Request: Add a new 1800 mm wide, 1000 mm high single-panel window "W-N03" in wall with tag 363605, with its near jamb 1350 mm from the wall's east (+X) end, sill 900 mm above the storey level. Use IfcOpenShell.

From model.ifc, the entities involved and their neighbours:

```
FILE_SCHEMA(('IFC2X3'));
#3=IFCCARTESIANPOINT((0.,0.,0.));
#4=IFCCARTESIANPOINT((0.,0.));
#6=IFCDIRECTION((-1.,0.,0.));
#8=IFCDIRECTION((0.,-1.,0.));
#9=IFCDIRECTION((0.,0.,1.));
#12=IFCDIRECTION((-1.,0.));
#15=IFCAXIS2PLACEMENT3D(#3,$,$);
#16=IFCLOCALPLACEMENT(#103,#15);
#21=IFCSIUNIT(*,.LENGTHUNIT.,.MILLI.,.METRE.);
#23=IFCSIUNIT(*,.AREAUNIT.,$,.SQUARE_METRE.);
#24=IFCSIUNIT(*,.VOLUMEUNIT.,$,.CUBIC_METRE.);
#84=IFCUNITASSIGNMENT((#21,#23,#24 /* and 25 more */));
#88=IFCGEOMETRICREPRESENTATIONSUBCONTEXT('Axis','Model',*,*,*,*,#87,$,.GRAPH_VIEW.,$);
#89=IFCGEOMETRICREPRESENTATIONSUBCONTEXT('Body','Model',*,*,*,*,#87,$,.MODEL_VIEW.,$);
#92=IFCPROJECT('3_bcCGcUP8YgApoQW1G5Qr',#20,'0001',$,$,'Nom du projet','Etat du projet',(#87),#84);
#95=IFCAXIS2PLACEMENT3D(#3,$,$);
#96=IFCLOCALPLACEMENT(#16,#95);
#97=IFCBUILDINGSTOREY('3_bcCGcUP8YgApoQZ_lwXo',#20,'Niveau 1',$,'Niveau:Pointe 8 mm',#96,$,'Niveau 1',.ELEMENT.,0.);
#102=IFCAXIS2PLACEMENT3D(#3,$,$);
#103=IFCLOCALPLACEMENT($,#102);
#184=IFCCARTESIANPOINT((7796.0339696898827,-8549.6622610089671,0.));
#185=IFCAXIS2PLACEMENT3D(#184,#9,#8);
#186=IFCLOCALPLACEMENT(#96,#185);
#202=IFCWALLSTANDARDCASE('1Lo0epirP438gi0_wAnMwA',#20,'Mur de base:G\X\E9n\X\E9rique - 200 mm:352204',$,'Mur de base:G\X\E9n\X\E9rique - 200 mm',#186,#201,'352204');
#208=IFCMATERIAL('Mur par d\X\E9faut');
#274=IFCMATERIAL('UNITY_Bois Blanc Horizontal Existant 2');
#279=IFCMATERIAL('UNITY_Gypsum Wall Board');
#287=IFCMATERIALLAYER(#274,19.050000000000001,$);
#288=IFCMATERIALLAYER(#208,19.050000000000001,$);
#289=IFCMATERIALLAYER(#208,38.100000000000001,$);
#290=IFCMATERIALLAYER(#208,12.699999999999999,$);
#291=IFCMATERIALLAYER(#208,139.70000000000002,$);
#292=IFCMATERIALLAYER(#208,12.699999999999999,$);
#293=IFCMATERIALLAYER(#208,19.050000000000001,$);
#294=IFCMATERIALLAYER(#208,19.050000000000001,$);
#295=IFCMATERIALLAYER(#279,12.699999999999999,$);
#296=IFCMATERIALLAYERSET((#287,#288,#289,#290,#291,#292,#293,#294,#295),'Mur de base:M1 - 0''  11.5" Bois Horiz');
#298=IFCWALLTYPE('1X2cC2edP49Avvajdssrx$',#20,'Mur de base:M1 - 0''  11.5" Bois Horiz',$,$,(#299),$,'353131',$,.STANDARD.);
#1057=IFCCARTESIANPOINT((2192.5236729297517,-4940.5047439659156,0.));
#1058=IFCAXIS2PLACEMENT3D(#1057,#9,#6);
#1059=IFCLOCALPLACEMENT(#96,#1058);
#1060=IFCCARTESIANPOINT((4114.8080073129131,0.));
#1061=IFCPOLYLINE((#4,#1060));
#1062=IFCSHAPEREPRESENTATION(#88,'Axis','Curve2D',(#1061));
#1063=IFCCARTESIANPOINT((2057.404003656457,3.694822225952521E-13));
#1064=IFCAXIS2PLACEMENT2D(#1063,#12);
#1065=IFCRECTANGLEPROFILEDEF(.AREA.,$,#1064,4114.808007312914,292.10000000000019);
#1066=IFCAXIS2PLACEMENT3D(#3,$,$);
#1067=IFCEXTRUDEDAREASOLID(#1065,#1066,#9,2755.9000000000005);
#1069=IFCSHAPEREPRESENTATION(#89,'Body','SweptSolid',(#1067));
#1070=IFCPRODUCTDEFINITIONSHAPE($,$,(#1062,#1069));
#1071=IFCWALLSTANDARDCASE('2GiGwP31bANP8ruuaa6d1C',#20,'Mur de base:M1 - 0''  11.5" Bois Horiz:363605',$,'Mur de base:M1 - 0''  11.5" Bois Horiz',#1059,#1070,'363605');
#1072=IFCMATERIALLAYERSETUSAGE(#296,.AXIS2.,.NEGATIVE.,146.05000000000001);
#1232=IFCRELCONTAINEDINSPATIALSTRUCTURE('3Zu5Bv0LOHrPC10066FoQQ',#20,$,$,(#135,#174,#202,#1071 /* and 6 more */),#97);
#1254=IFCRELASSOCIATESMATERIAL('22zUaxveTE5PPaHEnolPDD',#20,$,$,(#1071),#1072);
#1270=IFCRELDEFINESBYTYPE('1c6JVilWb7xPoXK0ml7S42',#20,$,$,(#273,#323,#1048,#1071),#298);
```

```python
import numpy as np
import ifcopenshell
import ifcopenshell.api.feature
import ifcopenshell.api.geometry
import ifcopenshell.api.root
import ifcopenshell.api.spatial
import ifcopenshell.api.type
import ifcopenshell.geom
import ifcopenshell.util.element
import ifcopenshell.util.placement
import ifcopenshell.util.representation
import ifcopenshell.util.shape
import ifcopenshell.util.unit

model = ifcopenshell.open("model.ifc")
unit_scale = ifcopenshell.util.unit.calculate_unit_scale(model)
settings = ifcopenshell.geom.settings()


def volume(element):
    """Net volume in cubic metres, openings subtracted."""
    shape = ifcopenshell.geom.create_shape(settings, element)
    return ifcopenshell.util.shape.get_volume(shape.geometry)


wall = model.by_guid("2GiGwP31bANP8ruuaa6d1C")
storey = ifcopenshell.util.element.get_container(wall, ifc_class="IfcBuildingStorey")
context = ifcopenshell.util.representation.get_context(model, "Model", "Body", "MODEL_VIEW")
before = volume(wall)

width, height, from_end, sill = 1.8, 1, 1.35, 0.9  # metres

# The wall runs along its own X axis, and the end named is its -X end.
wall_shape = ifcopenshell.geom.create_shape(settings, wall)
x, y, z = ifcopenshell.util.shape.get_vertices(wall_shape.geometry).T
start = x.min() + from_end
face, thickness = float(y.min()), float(y.max() - y.min())
wall_matrix = ifcopenshell.util.placement.get_local_placement(wall.ObjectPlacement)
level = ifcopenshell.util.placement.get_local_placement(storey.ObjectPlacement)[2, 3]


def in_wall(x, y):
    """Placement at x, y metres in the wall's axes, at sill height."""
    matrix = wall_matrix.copy()
    matrix[:, 3] = wall_matrix @ np.array([x / unit_scale, y / unit_scale, 0.0, 1.0])
    matrix[2, 3] = level + sill / unit_scale
    return matrix


# Opening: a box that overshoots both wall faces by 50 mm.
opening = ifcopenshell.api.root.create_entity(model, ifc_class="IfcOpeningElement")
box = ifcopenshell.api.geometry.add_wall_representation(
    model, context=context, length=width, height=height, thickness=thickness + 0.1
)
ifcopenshell.api.geometry.assign_representation(model, product=opening, representation=box)
ifcopenshell.api.geometry.edit_object_placement(model, product=opening, matrix=in_wall(start, face - 0.05), is_si=False)
ifcopenshell.api.feature.add_feature(model, feature=opening, element=wall)

window = ifcopenshell.api.root.create_entity(model, ifc_class="IfcWindow", name="W-N03")
window.OverallWidth, window.OverallHeight = width / unit_scale, height / unit_scale
body = ifcopenshell.api.geometry.add_window_representation(
    model,
    context=context,
    overall_width=window.OverallWidth,
    overall_height=window.OverallHeight,
    partition_type="SINGLE_PANEL",
)
ifcopenshell.api.geometry.assign_representation(model, product=window, representation=body)
ifcopenshell.api.spatial.assign_container(model, products=[window], relating_structure=storey)
fills = ifcopenshell.api.feature.add_filling(model, opening=opening, element=window)
fills.OwnerHistory = window.OwnerHistory  # required in IFC2X3

# IFC2X3 keeps the operation on the window style.
style = ifcopenshell.api.root.create_entity(model, ifc_class="IfcWindowStyle", name="W-N03")
style.OperationType, style.ConstructionType = "SINGLE_PANEL", "NOTDEFINED"
style.ParameterTakesPrecedence = style.Sizeable = False
ifcopenshell.api.type.assign_type(model, related_objects=[window], relating_type=style)

# Centre the window in the wall's thickness.
ifcopenshell.api.geometry.edit_object_placement(model, product=window, matrix=in_wall(start, face), is_si=False)
window_shape = ifcopenshell.geom.create_shape(settings, window)
depth = ifcopenshell.util.shape.get_vertices(window_shape.geometry)[:, 1]
offset = face + thickness / 2 - (depth.min() + depth.max()) / 2
ifcopenshell.api.geometry.edit_object_placement(model, product=window, matrix=in_wall(start, offset), is_si=False)

after = volume(wall)

print(f"wall volume {before:.3f} -> {after:.3f} m3")

model.write("model_updated.ifc")
```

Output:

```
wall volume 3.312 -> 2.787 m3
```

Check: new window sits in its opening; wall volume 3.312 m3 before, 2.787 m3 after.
